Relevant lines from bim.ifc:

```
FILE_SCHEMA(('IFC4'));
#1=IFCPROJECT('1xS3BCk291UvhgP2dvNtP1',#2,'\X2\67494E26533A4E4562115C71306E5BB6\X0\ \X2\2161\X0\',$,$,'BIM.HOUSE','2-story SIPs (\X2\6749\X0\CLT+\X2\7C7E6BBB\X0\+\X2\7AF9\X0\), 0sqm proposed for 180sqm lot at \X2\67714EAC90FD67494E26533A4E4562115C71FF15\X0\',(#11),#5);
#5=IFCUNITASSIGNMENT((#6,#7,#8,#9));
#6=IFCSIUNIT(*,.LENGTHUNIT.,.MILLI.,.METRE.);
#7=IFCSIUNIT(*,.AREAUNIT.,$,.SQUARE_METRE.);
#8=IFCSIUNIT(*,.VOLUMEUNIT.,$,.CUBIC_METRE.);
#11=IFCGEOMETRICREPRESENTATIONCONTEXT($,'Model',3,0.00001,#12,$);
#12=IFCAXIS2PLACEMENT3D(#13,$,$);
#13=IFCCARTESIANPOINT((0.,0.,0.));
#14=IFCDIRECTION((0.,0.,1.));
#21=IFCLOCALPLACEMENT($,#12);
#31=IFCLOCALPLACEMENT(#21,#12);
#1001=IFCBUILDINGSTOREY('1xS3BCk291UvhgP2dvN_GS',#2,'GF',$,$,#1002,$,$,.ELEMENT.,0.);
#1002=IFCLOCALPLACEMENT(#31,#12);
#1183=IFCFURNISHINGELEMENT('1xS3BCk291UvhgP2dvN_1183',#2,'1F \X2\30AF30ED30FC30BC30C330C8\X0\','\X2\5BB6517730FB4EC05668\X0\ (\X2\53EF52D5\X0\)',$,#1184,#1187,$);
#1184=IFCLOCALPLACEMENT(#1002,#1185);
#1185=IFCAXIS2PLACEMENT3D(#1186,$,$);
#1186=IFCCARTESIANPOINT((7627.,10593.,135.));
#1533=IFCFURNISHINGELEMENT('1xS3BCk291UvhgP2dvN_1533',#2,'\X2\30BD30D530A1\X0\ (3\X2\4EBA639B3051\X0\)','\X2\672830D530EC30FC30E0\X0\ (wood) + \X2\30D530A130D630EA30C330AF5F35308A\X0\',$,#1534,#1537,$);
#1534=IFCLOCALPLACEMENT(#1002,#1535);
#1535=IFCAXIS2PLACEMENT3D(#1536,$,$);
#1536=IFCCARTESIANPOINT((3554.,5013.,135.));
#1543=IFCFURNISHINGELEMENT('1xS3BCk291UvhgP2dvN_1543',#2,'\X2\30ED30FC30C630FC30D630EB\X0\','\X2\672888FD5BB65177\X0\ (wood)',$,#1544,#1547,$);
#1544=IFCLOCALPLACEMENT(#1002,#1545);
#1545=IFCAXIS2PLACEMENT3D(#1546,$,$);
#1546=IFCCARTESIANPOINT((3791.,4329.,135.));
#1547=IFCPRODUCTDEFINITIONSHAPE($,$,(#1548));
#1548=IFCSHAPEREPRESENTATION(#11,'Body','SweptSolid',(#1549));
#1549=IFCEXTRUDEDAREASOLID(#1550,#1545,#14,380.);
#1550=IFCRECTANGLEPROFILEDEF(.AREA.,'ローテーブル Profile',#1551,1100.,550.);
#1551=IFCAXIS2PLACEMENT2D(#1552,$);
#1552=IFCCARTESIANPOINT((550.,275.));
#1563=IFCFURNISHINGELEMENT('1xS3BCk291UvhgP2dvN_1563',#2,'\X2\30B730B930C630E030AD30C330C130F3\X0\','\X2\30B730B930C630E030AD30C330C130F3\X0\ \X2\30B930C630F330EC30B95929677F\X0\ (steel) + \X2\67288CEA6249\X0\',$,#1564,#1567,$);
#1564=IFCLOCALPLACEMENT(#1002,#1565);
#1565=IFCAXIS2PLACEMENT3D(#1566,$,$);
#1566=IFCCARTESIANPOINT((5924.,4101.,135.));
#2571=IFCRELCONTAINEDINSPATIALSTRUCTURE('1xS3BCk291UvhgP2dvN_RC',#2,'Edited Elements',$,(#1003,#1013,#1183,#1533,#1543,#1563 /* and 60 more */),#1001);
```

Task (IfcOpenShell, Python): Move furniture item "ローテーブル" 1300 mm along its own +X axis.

```python
import ifcopenshell
import ifcopenshell.api.geometry
import ifcopenshell.util.placement
import ifcopenshell.util.unit

model = ifcopenshell.open("bim.ifc")
unit_scale = ifcopenshell.util.unit.calculate_unit_scale(model)

item = model.by_guid("1xS3BCk291UvhgP2dvN_1543")
matrix = ifcopenshell.util.placement.get_local_placement(item.ObjectPlacement)
matrix[:3, 3] += matrix[:3, 0] * 1.3 / unit_scale
ifcopenshell.api.geometry.edit_object_placement(model, product=item, matrix=matrix, is_si=False)

print(ifcopenshell.util.placement.get_local_placement(item.ObjectPlacement).round(3) + 0.0)

model.write("bim-out.ifc")
```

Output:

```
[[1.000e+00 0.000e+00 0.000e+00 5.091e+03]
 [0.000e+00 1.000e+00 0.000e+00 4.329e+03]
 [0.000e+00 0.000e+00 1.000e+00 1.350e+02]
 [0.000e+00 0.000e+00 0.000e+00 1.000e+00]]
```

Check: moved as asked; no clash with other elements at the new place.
